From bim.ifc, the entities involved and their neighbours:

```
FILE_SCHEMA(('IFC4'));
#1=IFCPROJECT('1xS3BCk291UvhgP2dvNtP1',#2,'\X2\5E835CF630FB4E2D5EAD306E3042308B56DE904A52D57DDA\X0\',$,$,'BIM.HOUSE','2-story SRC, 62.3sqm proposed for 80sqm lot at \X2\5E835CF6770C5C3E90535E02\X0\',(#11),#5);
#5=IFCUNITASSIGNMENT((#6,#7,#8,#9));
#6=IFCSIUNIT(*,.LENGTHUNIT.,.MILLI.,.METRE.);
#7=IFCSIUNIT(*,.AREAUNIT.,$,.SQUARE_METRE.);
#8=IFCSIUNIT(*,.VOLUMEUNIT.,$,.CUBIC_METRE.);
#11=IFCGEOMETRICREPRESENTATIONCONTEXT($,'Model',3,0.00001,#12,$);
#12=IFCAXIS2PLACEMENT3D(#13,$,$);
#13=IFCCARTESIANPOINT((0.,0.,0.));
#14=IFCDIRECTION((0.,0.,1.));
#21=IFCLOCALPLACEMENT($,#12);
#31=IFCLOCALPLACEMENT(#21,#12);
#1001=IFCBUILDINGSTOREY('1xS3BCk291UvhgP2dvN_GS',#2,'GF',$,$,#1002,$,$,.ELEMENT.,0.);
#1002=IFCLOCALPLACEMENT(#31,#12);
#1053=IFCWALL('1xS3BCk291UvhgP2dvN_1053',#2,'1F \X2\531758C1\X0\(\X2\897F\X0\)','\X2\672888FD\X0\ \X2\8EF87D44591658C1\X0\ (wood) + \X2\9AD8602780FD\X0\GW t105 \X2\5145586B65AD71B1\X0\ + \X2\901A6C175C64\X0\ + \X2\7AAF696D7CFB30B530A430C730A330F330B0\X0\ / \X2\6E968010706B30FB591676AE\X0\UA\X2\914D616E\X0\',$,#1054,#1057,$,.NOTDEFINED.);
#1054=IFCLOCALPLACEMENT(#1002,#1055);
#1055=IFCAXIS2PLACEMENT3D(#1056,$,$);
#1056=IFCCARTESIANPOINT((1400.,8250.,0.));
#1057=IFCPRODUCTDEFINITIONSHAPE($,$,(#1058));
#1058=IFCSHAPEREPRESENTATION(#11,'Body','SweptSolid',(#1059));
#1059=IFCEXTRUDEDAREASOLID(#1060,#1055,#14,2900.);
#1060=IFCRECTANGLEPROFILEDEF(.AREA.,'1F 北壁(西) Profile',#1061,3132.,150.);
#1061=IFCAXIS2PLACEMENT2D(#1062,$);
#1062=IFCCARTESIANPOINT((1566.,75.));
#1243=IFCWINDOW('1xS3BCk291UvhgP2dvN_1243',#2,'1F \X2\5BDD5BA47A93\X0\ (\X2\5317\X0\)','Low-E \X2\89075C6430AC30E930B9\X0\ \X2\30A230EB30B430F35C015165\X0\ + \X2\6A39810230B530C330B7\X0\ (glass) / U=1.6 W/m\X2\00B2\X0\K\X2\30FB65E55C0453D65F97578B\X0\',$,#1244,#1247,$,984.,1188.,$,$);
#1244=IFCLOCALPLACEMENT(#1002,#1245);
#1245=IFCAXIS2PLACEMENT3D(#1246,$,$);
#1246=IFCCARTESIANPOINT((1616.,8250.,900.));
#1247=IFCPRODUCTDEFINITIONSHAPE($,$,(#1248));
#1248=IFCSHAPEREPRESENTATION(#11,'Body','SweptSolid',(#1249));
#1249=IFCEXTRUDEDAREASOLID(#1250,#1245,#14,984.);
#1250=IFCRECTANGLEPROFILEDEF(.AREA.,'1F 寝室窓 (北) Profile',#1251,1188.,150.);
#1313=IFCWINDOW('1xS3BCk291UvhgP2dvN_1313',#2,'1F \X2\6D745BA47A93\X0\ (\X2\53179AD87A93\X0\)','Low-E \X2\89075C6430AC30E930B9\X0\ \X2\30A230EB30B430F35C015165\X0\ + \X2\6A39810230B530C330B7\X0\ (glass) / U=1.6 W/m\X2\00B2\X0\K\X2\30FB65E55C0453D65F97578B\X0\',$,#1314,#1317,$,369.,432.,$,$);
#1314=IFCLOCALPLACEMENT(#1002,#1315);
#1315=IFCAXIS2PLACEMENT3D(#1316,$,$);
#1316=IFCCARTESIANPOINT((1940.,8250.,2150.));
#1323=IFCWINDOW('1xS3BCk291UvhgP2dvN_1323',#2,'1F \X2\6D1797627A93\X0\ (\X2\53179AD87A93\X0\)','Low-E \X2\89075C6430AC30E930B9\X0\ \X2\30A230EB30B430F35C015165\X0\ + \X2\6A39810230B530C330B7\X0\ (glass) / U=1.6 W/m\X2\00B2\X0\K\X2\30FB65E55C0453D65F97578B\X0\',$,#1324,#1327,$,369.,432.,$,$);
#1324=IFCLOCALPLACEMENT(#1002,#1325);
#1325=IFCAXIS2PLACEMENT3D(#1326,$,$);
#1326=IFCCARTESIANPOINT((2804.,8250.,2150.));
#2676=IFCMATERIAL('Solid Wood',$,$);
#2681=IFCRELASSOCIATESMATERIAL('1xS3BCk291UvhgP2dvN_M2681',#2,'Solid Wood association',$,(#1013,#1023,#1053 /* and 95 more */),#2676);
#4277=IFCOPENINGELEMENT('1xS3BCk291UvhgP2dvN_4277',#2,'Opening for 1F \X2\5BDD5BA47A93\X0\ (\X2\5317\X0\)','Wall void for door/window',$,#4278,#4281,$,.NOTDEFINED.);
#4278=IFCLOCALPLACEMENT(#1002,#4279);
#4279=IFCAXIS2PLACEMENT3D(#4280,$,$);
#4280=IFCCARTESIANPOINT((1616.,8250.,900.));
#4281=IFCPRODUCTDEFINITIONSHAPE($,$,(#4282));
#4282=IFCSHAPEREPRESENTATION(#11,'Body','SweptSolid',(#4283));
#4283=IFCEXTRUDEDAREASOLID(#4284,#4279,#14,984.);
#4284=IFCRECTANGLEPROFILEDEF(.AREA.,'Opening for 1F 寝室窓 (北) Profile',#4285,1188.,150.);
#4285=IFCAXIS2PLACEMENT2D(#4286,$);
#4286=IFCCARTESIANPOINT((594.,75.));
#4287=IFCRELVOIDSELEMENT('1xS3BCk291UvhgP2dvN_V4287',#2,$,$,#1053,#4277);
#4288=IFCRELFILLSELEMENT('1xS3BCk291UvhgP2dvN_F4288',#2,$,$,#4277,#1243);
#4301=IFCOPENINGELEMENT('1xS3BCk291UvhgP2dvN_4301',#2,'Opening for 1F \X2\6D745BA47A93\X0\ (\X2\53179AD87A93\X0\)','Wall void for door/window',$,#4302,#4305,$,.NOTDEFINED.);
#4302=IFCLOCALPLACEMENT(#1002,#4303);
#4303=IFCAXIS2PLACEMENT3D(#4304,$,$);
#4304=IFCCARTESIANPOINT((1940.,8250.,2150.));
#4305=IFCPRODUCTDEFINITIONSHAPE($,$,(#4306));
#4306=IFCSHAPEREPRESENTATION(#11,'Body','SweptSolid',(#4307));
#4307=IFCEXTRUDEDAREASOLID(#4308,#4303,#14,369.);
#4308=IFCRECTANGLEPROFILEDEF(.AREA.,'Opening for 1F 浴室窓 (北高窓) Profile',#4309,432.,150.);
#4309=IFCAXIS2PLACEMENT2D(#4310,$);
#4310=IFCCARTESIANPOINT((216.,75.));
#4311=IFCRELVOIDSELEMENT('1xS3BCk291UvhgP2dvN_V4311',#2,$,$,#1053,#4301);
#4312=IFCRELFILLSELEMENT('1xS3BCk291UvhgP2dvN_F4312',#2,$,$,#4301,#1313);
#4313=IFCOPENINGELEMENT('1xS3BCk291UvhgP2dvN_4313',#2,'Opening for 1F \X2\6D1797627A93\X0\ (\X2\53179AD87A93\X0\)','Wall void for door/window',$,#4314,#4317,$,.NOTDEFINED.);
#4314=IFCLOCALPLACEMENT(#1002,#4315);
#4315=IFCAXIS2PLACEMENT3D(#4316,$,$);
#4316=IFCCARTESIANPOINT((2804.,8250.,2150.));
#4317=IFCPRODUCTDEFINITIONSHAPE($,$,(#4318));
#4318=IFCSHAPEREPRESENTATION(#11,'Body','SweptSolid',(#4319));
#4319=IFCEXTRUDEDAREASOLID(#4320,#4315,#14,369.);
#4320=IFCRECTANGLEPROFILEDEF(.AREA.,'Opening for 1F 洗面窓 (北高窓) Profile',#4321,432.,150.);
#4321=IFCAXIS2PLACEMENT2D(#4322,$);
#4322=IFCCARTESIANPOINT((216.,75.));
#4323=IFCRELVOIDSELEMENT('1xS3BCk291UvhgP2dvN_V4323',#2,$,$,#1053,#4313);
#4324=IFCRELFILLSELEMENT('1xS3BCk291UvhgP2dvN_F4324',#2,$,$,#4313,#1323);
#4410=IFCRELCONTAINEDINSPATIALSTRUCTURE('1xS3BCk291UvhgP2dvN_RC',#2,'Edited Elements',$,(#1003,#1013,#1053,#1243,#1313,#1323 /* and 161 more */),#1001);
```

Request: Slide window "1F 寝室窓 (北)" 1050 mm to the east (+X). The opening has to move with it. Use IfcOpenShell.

```python
import ifcopenshell
import ifcopenshell.api.geometry
import ifcopenshell.util.placement

model = ifcopenshell.open("bim.ifc")

window = model.by_guid("1xS3BCk291UvhgP2dvN_1243")
opening = window.FillsVoids[0].RelatingOpeningElement
wall = opening.VoidsElements[0].RelatingBuildingElement

wall_matrix = ifcopenshell.util.placement.get_local_placement(wall.ObjectPlacement)
shift = wall_matrix[:3, 0] * 1050.0
before = ifcopenshell.util.placement.get_local_placement(window.ObjectPlacement)[:3, 3].copy()

# The window is not placed relative to its opening, so move both.
for product in (opening, window):
    matrix = ifcopenshell.util.placement.get_local_placement(product.ObjectPlacement)
    matrix[:3, 3] += shift
    ifcopenshell.api.geometry.edit_object_placement(model, product=product, matrix=matrix, is_si=False)

after = ifcopenshell.util.placement.get_local_placement(window.ObjectPlacement)[:3, 3]
print("window moved by", (after - before).round(3) + 0.0)

model.write("bim_rev.ifc")
```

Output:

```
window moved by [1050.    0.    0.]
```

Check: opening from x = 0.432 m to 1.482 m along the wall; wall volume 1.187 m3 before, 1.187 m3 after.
